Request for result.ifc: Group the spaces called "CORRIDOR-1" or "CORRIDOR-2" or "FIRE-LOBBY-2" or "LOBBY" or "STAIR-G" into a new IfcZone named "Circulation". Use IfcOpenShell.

First a look at what the model holds.

```python
import ifcopenshell

model = ifcopenshell.open("result.ifc")
print(model.schema)
seen = {}
for space in model.by_type("IfcSpace"):
    seen[space.Name] = seen.get(space.Name, 0) + 1
for name, count in sorted(seen.items(), key=str):
    print(count, "x", name)
print("zones:", [z.Name for z in model.by_type("IfcZone")][:20])
```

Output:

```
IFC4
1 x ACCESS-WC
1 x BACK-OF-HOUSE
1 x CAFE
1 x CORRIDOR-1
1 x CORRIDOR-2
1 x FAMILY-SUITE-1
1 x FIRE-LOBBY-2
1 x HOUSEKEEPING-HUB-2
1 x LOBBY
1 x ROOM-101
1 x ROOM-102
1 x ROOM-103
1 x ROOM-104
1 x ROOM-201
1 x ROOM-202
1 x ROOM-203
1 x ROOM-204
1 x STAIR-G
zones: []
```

```python
import ifcopenshell
import ifcopenshell.api.group
import ifcopenshell.api.root

model = ifcopenshell.open("result.ifc")

names = {"CORRIDOR-1", "CORRIDOR-2", "FIRE-LOBBY-2", "LOBBY", "STAIR-G"}
spaces = [s for s in model.by_type("IfcSpace") if s.Name in names]

zone = ifcopenshell.api.root.create_entity(model, ifc_class="IfcZone", name="Circulation")
ifcopenshell.api.group.assign_group(model, products=spaces, group=zone)
print(len(spaces), "spaces in", zone.Name)

model.write("result_edited.ifc")
```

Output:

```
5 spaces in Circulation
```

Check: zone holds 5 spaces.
